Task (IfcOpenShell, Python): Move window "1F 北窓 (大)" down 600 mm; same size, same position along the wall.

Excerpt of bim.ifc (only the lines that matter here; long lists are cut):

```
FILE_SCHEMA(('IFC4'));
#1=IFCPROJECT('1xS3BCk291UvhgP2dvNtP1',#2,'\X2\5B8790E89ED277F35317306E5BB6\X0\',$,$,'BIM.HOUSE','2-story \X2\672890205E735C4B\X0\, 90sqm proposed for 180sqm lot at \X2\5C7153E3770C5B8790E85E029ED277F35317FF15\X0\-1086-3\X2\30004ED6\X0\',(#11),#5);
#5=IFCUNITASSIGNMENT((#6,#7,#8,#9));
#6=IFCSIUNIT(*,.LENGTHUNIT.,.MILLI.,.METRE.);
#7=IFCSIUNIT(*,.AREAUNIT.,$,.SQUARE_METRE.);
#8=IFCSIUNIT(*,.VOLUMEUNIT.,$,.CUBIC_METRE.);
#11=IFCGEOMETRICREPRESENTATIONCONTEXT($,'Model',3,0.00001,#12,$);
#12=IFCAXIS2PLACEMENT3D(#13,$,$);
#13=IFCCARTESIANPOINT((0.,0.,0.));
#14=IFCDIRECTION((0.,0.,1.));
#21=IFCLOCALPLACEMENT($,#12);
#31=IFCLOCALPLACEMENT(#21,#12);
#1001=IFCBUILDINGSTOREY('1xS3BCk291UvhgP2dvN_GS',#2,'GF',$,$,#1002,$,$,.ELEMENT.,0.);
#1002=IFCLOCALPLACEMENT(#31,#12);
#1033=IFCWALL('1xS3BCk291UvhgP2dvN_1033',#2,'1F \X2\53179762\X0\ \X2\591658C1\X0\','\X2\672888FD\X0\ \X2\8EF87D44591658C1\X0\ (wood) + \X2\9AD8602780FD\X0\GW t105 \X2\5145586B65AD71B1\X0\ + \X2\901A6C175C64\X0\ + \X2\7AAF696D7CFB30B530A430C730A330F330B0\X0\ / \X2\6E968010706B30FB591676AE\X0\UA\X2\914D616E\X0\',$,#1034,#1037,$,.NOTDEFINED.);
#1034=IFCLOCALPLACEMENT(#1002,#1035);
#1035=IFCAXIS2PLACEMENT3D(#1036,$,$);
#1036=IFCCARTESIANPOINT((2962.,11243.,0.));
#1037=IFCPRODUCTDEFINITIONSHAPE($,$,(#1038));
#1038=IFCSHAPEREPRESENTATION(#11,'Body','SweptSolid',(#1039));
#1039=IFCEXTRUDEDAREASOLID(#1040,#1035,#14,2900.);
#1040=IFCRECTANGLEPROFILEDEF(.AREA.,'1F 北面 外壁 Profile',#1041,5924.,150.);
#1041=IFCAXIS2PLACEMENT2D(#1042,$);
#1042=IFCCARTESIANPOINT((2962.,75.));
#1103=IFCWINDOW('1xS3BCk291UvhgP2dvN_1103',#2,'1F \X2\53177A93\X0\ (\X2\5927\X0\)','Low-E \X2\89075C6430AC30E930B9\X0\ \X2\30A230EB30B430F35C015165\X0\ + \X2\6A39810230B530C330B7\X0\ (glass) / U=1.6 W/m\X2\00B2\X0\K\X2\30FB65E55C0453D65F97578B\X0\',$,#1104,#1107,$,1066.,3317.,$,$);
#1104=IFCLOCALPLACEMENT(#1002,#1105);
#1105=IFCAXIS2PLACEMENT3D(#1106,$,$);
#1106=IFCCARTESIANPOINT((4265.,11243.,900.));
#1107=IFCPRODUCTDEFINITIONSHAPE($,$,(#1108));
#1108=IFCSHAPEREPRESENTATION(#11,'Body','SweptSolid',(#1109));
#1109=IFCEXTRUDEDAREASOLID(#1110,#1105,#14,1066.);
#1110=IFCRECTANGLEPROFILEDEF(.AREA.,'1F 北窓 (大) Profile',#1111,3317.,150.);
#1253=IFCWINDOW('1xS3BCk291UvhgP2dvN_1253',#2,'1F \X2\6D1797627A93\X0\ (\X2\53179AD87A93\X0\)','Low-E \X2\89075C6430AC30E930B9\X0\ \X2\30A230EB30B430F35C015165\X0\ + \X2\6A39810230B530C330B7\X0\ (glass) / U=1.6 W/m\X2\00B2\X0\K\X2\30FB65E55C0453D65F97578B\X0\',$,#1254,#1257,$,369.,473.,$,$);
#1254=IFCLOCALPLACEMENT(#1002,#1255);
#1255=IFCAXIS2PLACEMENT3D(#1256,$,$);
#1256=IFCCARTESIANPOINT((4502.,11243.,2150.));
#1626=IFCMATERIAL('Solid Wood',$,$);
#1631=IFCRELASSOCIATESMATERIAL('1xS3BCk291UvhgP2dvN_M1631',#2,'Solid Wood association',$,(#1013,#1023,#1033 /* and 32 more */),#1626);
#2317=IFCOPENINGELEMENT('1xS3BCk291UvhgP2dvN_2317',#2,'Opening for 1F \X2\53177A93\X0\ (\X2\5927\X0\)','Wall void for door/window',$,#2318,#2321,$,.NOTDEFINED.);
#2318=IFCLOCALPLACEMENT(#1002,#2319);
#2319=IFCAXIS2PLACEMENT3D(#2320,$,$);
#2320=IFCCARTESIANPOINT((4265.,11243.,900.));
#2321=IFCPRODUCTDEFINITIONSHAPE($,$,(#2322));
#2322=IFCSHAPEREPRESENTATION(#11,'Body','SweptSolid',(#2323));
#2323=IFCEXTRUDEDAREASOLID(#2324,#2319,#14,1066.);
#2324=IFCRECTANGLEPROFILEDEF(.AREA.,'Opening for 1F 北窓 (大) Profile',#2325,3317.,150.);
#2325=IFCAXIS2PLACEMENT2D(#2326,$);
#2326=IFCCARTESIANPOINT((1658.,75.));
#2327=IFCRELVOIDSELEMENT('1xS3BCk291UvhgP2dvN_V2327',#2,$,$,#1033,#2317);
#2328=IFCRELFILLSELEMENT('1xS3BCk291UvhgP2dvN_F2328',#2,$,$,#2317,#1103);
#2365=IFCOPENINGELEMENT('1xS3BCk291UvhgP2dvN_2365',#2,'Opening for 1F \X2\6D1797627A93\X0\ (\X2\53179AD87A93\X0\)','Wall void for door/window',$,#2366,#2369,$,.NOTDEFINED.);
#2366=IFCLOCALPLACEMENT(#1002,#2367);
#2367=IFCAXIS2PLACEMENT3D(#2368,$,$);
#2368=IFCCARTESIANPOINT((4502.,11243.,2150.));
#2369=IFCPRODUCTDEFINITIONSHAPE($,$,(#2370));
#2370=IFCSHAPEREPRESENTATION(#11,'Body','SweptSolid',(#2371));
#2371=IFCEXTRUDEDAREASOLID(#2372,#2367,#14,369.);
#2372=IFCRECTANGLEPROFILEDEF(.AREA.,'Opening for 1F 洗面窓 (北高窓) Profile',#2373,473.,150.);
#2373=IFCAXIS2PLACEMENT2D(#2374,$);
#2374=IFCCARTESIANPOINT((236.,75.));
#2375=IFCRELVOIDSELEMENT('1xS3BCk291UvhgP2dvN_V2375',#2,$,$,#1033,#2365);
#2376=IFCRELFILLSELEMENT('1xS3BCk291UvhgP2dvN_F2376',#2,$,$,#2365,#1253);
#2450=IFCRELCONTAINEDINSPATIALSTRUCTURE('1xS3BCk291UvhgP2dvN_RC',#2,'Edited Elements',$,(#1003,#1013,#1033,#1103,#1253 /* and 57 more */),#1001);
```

```python
import numpy as np
import ifcopenshell
import ifcopenshell.api.geometry
import ifcopenshell.util.placement
import ifcopenshell.util.unit

model = ifcopenshell.open("bim.ifc")
unit_scale = ifcopenshell.util.unit.calculate_unit_scale(model)

window = model.by_id(1103)
opening = window.FillsVoids[0].RelatingOpeningElement
dz = -600.0

shift = np.array([0.0, 0.0, dz])
# The window is not placed relative to its opening, so move both.
for product in (opening, window):
    matrix = ifcopenshell.util.placement.get_local_placement(product.ObjectPlacement)
    matrix[:3, 3] += shift
    ifcopenshell.api.geometry.edit_object_placement(model, product=product, matrix=matrix, is_si=False)

print(f"moved by {dz * unit_scale:+.3f} m")

model.write("bim_rev.ifc")
```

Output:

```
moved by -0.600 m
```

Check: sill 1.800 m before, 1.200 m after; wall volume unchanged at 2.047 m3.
